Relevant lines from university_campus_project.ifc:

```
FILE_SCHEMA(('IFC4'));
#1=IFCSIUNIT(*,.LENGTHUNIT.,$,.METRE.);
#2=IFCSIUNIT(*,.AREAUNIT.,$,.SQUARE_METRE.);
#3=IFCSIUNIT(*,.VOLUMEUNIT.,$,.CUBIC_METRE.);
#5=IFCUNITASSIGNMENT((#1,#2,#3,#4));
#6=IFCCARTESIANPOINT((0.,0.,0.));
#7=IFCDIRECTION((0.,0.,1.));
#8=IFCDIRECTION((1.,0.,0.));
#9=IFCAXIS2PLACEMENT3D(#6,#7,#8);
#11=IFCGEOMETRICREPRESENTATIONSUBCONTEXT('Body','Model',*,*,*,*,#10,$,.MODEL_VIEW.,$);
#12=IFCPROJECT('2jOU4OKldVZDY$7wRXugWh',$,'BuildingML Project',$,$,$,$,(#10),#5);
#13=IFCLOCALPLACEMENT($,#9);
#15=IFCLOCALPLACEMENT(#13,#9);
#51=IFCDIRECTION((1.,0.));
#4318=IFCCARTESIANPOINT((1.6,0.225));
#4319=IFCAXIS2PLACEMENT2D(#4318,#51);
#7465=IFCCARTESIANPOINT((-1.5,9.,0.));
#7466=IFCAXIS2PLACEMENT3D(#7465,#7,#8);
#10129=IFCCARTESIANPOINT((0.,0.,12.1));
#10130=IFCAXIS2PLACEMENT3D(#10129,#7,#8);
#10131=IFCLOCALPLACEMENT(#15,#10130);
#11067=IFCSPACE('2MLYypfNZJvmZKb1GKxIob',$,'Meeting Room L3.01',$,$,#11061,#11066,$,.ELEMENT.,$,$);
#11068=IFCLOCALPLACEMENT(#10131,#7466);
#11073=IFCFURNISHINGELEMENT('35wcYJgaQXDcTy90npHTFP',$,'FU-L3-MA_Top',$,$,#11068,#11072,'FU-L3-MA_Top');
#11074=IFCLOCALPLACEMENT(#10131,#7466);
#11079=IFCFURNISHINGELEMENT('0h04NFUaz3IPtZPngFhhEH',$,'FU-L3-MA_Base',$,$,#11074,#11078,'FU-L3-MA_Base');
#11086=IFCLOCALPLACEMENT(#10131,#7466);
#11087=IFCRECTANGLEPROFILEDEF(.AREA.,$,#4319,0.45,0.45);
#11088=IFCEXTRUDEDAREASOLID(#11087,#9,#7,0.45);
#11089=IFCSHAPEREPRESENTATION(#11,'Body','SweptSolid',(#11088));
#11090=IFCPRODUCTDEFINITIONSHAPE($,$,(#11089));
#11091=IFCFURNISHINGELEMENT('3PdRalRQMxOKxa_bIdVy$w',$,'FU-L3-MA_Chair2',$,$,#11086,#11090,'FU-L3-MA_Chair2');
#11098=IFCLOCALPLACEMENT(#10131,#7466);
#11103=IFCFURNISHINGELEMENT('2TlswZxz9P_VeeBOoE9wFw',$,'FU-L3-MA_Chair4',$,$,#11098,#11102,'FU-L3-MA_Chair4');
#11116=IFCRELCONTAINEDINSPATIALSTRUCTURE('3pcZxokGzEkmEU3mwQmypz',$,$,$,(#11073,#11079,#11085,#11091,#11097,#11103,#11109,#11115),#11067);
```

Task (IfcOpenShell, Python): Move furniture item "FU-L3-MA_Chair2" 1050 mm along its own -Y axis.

```python
import ifcopenshell
import ifcopenshell.api.geometry
import ifcopenshell.util.placement
import ifcopenshell.util.unit

model = ifcopenshell.open("university_campus_project.ifc")
unit_scale = ifcopenshell.util.unit.calculate_unit_scale(model)

item = model.by_guid("3PdRalRQMxOKxa_bIdVy$w")
matrix = ifcopenshell.util.placement.get_local_placement(item.ObjectPlacement)
matrix[:3, 3] -= matrix[:3, 1] * 1.05 / unit_scale
ifcopenshell.api.geometry.edit_object_placement(model, product=item, matrix=matrix, is_si=False)

print(ifcopenshell.util.placement.get_local_placement(item.ObjectPlacement).round(3) + 0.0)

model.write("university_campus_project_updated.ifc")
```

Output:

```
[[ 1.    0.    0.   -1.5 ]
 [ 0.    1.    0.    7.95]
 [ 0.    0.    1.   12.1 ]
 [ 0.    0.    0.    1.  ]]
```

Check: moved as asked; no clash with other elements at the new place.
